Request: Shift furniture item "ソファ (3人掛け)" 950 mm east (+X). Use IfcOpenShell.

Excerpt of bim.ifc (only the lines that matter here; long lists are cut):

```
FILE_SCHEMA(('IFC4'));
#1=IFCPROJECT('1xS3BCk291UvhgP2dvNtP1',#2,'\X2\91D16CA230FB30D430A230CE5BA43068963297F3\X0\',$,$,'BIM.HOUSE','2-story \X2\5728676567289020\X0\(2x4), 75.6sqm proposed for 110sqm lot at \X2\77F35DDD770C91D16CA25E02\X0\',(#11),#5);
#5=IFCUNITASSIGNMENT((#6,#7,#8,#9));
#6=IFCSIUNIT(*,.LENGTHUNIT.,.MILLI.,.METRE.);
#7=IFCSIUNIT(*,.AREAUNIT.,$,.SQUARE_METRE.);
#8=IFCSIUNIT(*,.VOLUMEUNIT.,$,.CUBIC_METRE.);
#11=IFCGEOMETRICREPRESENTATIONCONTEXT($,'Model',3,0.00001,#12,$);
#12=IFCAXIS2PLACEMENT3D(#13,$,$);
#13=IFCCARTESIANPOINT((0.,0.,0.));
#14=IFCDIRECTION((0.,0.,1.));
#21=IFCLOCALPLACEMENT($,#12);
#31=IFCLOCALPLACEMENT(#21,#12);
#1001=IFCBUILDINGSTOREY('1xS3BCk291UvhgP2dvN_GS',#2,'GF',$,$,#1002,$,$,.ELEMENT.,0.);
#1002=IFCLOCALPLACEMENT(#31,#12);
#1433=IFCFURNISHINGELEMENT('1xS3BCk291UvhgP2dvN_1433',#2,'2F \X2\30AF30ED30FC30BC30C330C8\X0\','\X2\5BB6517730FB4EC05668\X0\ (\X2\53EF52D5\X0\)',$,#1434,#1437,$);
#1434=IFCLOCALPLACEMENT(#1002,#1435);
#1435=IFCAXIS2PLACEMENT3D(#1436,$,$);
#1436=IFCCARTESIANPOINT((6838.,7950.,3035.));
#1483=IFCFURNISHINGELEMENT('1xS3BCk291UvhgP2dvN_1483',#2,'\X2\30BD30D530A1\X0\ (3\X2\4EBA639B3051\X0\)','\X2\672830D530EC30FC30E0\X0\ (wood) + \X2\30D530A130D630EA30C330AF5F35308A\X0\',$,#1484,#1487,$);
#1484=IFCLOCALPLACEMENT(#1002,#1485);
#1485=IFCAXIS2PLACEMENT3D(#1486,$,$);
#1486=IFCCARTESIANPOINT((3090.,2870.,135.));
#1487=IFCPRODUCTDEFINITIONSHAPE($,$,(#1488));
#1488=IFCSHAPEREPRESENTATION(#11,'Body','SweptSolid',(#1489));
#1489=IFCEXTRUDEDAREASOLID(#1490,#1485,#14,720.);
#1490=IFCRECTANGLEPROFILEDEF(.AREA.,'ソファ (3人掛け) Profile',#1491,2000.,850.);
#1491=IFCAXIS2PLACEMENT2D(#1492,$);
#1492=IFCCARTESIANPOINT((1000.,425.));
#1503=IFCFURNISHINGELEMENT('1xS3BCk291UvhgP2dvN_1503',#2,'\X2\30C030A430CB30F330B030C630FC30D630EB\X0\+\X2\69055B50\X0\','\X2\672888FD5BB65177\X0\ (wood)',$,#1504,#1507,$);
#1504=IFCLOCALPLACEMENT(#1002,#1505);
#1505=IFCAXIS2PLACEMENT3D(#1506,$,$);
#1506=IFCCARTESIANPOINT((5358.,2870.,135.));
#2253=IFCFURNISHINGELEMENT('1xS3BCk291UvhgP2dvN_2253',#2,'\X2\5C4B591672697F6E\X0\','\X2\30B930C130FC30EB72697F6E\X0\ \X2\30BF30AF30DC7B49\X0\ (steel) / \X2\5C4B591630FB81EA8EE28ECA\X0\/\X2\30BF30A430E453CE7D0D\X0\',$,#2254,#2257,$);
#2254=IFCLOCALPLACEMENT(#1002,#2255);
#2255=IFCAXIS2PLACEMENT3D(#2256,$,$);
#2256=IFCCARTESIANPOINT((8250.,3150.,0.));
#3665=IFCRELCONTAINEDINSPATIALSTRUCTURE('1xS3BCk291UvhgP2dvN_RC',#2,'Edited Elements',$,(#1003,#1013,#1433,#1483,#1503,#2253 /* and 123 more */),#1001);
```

```python
import ifcopenshell
import ifcopenshell.api.geometry
import ifcopenshell.util.placement
import ifcopenshell.util.unit

model = ifcopenshell.open("bim.ifc")
unit_scale = ifcopenshell.util.unit.calculate_unit_scale(model)

item = model.by_guid("1xS3BCk291UvhgP2dvN_1483")
matrix = ifcopenshell.util.placement.get_local_placement(item.ObjectPlacement)
matrix[0, 3] += 0.95 / unit_scale
ifcopenshell.api.geometry.edit_object_placement(model, product=item, matrix=matrix, is_si=False)

print(ifcopenshell.util.placement.get_local_placement(item.ObjectPlacement).round(3) + 0.0)

model.write("bim-out.ifc")
```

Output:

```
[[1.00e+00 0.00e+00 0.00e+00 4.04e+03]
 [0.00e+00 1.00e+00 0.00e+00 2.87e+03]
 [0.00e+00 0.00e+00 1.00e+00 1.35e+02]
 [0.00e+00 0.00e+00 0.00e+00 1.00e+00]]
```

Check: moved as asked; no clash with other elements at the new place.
